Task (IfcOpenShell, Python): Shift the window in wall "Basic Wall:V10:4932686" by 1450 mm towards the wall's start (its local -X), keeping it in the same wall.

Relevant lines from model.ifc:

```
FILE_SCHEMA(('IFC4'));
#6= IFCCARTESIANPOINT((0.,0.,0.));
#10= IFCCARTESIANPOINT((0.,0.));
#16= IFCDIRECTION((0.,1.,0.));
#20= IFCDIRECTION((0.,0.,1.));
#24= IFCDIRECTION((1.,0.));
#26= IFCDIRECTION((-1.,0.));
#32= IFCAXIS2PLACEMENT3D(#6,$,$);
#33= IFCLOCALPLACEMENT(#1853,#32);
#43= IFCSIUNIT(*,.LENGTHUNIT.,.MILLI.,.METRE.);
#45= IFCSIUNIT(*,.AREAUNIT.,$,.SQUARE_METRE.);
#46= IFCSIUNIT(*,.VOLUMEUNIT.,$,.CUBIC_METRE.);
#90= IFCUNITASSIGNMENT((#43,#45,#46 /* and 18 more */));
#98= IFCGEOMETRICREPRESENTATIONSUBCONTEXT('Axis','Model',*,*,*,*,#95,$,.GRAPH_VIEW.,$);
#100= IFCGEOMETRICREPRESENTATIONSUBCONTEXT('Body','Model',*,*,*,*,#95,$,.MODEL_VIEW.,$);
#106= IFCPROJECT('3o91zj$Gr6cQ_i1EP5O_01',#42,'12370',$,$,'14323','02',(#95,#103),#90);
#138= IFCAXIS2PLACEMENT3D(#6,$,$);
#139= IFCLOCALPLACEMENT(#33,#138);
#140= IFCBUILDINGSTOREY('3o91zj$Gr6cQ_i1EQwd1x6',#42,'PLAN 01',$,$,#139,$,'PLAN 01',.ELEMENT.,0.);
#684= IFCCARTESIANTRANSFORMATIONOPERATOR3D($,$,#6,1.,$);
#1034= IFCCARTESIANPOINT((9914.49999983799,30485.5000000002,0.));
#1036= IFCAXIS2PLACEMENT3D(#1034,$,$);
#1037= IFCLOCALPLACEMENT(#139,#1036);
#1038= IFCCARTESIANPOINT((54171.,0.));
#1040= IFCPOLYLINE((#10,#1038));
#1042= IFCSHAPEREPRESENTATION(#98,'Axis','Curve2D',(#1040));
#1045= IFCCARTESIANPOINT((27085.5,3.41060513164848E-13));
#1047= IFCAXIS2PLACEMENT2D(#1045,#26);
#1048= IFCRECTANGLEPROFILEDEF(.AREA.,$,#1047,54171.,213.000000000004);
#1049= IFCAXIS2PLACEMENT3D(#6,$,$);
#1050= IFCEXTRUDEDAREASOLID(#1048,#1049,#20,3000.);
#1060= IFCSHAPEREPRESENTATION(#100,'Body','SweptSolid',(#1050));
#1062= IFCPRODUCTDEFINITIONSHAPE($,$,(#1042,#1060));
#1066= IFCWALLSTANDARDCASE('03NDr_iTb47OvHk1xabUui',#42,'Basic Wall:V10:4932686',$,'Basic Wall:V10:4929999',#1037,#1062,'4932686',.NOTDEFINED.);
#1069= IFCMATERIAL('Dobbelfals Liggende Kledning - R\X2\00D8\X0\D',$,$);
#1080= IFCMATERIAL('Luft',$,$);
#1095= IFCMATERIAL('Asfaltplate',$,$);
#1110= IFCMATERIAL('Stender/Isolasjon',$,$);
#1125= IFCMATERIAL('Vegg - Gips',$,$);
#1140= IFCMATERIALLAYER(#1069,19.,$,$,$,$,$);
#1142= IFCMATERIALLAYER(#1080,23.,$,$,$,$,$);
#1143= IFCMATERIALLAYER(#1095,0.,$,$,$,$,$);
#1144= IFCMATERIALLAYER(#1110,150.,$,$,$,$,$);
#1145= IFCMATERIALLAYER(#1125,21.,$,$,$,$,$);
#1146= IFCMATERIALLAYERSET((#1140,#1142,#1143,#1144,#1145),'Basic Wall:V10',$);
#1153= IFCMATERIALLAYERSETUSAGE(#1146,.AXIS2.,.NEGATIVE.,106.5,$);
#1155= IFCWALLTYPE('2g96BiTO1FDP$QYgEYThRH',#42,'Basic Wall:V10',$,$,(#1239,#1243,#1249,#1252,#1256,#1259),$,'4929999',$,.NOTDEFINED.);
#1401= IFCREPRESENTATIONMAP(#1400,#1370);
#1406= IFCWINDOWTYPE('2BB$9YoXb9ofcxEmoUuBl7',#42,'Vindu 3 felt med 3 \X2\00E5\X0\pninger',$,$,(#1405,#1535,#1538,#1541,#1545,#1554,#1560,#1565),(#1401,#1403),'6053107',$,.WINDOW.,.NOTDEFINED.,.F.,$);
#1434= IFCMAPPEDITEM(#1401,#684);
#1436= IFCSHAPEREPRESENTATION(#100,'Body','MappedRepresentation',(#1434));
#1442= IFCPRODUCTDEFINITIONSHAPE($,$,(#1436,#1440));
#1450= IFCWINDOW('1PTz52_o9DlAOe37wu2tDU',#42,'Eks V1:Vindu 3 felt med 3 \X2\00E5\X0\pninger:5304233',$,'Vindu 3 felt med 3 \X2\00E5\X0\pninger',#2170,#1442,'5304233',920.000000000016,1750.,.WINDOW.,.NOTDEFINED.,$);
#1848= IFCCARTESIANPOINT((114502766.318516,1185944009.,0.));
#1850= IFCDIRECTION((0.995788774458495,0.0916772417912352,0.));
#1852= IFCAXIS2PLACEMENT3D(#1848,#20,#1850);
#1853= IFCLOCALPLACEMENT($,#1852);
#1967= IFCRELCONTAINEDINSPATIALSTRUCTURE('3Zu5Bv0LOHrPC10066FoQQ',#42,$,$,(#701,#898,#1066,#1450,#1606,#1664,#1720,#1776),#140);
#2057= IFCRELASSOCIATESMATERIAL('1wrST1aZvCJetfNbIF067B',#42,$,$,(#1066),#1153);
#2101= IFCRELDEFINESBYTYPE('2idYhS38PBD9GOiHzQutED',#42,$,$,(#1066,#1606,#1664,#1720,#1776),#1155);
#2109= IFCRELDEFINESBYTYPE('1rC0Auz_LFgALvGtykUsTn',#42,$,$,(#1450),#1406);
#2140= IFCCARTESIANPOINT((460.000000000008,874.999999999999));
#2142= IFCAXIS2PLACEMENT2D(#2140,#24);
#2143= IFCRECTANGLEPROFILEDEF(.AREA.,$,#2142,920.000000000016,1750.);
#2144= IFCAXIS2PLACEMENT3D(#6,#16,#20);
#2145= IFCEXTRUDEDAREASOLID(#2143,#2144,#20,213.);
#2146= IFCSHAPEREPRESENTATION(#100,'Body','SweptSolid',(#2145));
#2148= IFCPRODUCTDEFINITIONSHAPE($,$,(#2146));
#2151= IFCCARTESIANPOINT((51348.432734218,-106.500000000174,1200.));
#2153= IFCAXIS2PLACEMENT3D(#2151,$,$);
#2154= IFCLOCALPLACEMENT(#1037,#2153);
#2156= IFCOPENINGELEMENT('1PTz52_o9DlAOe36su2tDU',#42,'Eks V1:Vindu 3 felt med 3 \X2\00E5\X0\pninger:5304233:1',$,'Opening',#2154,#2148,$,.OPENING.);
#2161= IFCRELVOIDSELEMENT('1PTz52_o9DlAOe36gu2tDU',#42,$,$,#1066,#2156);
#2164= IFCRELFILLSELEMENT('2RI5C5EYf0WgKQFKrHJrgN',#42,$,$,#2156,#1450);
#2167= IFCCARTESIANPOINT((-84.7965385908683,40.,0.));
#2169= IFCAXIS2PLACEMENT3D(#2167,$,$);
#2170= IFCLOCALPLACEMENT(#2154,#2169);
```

```python
import ifcopenshell
import ifcopenshell.api.geometry
import ifcopenshell.util.placement
import ifcopenshell.util.unit

model = ifcopenshell.open("model.ifc")
unit_scale = ifcopenshell.util.unit.calculate_unit_scale(model)

window = model.by_guid("1PTz52_o9DlAOe37wu2tDU")
opening = window.FillsVoids[0].RelatingOpeningElement
wall = opening.VoidsElements[0].RelatingBuildingElement

wall_matrix = ifcopenshell.util.placement.get_local_placement(wall.ObjectPlacement)
shift = wall_matrix[:3, 0] * -1.45 / unit_scale
before = ifcopenshell.util.placement.get_local_placement(window.ObjectPlacement)[:3, 3].copy()

# The window is placed relative to its opening, so it follows when the opening moves.
matrix = ifcopenshell.util.placement.get_local_placement(opening.ObjectPlacement)
matrix[:3, 3] += shift
ifcopenshell.api.geometry.edit_object_placement(
    model, product=opening, matrix=matrix, is_si=False, should_transform_children=True
)

after = ifcopenshell.util.placement.get_local_placement(window.ObjectPlacement)[:3, 3]
print("window moved by", (after - before).round(3) + 0.0)

model.write("model_edited.ifc")
```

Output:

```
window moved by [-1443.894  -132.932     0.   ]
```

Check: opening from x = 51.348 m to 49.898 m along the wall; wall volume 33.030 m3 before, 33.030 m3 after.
